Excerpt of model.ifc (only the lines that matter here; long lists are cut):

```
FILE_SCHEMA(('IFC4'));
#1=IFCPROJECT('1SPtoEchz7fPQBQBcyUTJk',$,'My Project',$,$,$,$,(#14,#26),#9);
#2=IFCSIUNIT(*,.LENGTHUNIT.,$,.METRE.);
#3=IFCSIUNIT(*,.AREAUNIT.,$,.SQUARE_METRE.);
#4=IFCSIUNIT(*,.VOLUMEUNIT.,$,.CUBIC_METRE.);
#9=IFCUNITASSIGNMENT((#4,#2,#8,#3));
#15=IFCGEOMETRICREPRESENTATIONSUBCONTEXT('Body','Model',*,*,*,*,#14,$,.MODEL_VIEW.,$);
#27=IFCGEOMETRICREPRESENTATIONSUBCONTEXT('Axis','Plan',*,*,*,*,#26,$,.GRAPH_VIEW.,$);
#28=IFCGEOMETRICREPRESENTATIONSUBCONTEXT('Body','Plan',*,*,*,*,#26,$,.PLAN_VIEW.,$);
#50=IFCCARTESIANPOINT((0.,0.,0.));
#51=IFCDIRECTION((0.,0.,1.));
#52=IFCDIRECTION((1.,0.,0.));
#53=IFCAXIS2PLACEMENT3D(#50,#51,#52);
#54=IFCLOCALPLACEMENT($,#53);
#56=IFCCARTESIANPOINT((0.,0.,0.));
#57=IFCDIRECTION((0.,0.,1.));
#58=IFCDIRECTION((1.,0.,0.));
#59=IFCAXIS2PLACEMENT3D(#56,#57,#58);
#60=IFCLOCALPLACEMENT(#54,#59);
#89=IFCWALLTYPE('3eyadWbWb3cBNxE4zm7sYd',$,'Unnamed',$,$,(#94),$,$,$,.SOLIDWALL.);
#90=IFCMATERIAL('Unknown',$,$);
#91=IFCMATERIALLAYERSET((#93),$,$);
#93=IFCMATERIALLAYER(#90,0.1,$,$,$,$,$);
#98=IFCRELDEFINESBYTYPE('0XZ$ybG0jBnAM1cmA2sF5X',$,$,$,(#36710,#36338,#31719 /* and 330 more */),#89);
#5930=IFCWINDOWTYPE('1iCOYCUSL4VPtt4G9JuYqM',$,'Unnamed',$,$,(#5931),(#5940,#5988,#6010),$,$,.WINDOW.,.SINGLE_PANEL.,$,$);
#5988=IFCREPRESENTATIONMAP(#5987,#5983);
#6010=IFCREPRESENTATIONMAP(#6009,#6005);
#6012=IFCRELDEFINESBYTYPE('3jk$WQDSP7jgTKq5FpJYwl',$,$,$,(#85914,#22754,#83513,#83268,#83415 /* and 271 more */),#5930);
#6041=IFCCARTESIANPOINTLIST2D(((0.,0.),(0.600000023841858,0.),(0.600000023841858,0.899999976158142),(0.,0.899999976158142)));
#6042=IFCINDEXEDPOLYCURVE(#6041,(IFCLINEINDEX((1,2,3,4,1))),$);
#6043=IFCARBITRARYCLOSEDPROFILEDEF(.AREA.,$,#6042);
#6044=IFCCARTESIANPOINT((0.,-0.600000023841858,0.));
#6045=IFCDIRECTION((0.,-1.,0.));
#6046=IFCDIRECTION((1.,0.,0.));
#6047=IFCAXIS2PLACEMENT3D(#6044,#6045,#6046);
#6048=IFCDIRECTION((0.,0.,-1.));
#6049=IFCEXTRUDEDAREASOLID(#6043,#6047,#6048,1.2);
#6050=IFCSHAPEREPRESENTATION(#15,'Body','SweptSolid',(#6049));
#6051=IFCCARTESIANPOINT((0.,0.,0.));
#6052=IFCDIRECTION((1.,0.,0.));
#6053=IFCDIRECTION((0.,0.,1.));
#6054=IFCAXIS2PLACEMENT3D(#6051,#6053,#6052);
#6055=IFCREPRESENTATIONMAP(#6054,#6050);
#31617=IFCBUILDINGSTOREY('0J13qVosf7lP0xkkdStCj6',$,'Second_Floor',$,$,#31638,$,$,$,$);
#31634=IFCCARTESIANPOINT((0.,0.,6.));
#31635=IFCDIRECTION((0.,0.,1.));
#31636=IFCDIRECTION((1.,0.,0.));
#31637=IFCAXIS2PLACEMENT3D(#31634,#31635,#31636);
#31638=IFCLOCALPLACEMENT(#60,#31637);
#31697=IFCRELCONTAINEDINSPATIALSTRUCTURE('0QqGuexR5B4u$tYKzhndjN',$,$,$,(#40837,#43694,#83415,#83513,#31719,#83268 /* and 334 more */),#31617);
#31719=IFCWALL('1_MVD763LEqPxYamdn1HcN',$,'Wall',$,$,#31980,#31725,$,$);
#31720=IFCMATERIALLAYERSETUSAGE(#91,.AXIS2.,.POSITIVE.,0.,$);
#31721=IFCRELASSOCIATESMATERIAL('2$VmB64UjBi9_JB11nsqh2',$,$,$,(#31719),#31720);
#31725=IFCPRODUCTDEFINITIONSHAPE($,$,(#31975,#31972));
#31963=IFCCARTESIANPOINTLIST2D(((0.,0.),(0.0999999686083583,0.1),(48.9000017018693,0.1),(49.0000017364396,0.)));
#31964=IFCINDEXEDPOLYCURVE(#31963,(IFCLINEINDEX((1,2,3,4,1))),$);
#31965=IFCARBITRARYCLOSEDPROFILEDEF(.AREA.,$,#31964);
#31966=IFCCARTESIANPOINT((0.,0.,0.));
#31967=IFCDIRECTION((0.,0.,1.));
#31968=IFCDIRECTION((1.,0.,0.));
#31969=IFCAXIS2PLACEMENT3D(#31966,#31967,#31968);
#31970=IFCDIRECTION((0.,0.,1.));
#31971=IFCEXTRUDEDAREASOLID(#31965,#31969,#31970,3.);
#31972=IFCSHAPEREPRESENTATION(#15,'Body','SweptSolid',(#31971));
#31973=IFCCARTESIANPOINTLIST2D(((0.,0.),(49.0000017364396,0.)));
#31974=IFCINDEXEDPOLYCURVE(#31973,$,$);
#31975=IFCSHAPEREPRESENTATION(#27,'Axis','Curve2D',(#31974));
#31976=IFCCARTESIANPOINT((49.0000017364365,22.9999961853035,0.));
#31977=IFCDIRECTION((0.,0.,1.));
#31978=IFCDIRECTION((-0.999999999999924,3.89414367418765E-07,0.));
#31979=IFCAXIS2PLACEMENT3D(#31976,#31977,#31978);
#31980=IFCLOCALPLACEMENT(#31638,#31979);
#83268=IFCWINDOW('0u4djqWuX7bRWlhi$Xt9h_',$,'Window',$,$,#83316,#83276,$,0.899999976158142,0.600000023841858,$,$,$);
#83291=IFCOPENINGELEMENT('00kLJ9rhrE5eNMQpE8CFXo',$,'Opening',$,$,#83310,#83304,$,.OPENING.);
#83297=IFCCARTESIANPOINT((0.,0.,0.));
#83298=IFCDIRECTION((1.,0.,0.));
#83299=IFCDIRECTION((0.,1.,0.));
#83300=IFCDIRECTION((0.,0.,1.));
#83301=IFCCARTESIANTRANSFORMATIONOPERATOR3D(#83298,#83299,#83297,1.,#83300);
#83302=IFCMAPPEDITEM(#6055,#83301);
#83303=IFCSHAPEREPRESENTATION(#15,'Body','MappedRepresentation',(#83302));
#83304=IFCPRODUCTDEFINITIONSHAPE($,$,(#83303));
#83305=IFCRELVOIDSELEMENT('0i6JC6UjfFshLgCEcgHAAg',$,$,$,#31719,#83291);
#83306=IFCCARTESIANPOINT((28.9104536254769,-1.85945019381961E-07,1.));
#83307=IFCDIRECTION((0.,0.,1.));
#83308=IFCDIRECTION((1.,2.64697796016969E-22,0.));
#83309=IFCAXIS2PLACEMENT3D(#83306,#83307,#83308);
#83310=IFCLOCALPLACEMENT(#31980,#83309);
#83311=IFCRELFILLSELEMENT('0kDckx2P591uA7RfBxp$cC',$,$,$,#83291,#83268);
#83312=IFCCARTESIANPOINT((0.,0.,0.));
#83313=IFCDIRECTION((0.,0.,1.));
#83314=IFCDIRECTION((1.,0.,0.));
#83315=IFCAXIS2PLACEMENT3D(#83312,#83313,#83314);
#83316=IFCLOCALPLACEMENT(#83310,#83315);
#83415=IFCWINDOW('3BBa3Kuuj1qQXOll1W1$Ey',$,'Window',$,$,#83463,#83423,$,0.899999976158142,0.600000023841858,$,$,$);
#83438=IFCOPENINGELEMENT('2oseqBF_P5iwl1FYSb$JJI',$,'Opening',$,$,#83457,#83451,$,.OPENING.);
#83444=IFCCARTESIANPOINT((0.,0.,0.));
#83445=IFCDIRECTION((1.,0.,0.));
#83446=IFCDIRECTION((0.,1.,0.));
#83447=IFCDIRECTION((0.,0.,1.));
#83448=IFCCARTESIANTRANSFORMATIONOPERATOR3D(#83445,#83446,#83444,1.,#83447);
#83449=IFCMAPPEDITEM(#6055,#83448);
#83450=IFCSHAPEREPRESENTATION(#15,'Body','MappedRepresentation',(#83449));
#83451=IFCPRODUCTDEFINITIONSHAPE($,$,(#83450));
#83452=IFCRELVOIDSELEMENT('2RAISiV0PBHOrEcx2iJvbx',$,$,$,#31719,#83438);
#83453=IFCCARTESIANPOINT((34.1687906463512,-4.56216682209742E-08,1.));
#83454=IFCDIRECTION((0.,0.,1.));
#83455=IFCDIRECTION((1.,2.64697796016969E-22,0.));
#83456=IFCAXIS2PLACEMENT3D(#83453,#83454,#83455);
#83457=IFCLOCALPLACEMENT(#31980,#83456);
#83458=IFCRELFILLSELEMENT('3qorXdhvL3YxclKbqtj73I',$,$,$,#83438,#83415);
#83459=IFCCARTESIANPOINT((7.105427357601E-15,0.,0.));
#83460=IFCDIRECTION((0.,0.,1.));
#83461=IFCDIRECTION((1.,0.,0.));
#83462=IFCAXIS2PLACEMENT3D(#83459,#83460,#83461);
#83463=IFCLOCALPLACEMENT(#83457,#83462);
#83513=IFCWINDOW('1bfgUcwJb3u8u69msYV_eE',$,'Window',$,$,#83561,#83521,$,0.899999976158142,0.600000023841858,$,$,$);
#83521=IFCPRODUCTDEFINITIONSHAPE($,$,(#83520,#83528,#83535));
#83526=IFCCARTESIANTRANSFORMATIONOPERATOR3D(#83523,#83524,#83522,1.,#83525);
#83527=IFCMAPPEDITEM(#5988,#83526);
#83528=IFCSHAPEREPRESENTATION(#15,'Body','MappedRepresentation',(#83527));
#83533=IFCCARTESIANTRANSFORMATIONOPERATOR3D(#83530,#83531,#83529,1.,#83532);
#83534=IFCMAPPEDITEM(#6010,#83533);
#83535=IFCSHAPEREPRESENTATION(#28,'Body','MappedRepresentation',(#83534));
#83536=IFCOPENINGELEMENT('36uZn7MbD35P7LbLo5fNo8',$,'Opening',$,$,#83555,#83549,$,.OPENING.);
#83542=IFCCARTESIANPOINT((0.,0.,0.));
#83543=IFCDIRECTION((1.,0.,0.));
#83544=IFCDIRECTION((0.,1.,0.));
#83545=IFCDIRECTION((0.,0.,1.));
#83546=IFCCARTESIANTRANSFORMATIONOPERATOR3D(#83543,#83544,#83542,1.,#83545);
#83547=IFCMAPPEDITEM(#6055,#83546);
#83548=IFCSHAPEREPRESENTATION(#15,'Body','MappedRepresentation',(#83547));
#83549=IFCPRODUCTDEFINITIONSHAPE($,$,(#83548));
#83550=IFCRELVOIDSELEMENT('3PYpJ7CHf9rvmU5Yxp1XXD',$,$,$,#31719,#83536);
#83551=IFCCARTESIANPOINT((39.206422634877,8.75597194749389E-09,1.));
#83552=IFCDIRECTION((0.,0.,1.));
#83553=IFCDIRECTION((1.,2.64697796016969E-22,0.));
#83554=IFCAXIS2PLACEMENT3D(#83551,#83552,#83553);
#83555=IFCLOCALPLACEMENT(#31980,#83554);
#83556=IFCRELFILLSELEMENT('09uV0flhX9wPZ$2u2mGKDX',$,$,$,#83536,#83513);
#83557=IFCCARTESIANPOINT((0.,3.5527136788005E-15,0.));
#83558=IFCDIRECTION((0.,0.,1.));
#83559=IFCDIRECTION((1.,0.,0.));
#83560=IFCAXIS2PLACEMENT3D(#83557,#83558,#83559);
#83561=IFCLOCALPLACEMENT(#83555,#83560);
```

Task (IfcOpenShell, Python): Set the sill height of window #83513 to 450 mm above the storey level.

```python
import numpy as np
import ifcopenshell
import ifcopenshell.api.geometry
import ifcopenshell.geom
import ifcopenshell.util.element
import ifcopenshell.util.placement
import ifcopenshell.util.shape
import ifcopenshell.util.unit

model = ifcopenshell.open("model.ifc")
unit_scale = ifcopenshell.util.unit.calculate_unit_scale(model)

window = model.by_guid("1bfgUcwJb3u8u69msYV_eE")
opening = window.FillsVoids[0].RelatingOpeningElement
storey = ifcopenshell.util.element.get_container(window, ifc_class="IfcBuildingStorey")
level = ifcopenshell.util.placement.get_local_placement(storey.ObjectPlacement)[2, 3]

# The opening's origin need not be at the sill, so measure its lowest point.
shape = ifcopenshell.geom.create_shape(ifcopenshell.geom.settings(), opening)
bottom = ifcopenshell.util.shape.get_shape_bottom_elevation(shape, shape.geometry) / unit_scale
dz = level + 0.45 - bottom

shift = np.array([0.0, 0.0, dz])
# The window is placed relative to its opening, so it follows when the opening moves.
matrix = ifcopenshell.util.placement.get_local_placement(opening.ObjectPlacement)
matrix[:3, 3] += shift
ifcopenshell.api.geometry.edit_object_placement(
    model, product=opening, matrix=matrix, is_si=False, should_transform_children=True
)

print(f"moved by {dz * unit_scale:+.3f} m")

model.write("model_v2.ifc")
```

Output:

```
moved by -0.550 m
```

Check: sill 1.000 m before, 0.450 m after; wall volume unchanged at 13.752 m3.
